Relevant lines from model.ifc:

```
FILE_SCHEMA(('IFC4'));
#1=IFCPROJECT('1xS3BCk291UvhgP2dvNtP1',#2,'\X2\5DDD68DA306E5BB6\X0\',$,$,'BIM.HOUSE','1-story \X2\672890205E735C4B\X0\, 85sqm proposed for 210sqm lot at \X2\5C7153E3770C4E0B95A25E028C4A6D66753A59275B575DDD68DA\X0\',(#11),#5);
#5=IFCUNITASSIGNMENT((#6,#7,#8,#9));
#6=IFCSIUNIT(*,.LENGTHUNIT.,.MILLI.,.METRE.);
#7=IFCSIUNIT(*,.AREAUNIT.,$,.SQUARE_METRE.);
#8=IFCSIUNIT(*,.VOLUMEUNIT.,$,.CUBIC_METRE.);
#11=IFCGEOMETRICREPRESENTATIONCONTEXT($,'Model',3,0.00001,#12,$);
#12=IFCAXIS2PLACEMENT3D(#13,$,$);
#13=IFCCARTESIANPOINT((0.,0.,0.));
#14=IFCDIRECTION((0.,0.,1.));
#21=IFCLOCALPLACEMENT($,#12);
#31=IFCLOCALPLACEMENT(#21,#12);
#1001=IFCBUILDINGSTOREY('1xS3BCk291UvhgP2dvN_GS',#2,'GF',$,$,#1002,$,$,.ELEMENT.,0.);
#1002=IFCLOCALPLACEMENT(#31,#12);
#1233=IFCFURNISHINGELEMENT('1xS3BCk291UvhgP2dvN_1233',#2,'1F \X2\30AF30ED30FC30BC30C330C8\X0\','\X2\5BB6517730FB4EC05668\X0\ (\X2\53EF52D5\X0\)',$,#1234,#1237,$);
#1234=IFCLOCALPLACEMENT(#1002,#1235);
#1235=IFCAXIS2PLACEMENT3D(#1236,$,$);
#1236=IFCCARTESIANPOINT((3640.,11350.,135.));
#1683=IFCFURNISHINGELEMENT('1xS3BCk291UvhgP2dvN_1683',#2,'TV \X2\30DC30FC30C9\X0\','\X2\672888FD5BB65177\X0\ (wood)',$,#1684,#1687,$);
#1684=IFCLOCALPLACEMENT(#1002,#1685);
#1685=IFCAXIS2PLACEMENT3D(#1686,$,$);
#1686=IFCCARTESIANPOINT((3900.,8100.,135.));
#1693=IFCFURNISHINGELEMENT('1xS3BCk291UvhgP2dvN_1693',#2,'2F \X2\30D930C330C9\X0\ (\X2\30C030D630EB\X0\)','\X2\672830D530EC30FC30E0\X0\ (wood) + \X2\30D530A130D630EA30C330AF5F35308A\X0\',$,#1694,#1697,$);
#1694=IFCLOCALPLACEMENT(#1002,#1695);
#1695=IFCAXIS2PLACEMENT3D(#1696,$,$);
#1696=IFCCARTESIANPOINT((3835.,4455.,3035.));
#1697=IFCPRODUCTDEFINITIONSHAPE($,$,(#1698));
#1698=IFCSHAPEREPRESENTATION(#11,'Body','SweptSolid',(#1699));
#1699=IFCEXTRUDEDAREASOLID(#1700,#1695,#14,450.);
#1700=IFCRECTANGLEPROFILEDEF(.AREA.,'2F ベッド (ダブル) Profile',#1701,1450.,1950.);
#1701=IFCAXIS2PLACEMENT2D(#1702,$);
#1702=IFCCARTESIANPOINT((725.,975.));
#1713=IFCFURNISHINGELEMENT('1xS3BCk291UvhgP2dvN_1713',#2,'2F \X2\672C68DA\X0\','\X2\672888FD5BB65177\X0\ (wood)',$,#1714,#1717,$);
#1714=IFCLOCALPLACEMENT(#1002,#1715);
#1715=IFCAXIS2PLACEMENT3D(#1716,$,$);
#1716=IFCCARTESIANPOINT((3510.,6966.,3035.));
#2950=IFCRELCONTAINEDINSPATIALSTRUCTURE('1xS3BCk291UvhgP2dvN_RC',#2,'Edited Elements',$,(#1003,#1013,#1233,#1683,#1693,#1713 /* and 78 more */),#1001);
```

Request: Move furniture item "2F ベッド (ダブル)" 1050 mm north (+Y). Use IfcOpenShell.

```python
import ifcopenshell
import ifcopenshell.api.geometry
import ifcopenshell.util.placement
import ifcopenshell.util.unit

model = ifcopenshell.open("model.ifc")
unit_scale = ifcopenshell.util.unit.calculate_unit_scale(model)

item = model.by_guid("1xS3BCk291UvhgP2dvN_1693")
matrix = ifcopenshell.util.placement.get_local_placement(item.ObjectPlacement)
matrix[1, 3] += 1.05 / unit_scale
ifcopenshell.api.geometry.edit_object_placement(model, product=item, matrix=matrix, is_si=False)

print(ifcopenshell.util.placement.get_local_placement(item.ObjectPlacement).round(3) + 0.0)

model.write("model_updated.ifc")
```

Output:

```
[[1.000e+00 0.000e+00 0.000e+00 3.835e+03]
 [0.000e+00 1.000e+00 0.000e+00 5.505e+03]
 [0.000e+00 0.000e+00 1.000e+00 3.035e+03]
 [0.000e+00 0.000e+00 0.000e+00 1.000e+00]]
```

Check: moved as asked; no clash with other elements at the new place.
